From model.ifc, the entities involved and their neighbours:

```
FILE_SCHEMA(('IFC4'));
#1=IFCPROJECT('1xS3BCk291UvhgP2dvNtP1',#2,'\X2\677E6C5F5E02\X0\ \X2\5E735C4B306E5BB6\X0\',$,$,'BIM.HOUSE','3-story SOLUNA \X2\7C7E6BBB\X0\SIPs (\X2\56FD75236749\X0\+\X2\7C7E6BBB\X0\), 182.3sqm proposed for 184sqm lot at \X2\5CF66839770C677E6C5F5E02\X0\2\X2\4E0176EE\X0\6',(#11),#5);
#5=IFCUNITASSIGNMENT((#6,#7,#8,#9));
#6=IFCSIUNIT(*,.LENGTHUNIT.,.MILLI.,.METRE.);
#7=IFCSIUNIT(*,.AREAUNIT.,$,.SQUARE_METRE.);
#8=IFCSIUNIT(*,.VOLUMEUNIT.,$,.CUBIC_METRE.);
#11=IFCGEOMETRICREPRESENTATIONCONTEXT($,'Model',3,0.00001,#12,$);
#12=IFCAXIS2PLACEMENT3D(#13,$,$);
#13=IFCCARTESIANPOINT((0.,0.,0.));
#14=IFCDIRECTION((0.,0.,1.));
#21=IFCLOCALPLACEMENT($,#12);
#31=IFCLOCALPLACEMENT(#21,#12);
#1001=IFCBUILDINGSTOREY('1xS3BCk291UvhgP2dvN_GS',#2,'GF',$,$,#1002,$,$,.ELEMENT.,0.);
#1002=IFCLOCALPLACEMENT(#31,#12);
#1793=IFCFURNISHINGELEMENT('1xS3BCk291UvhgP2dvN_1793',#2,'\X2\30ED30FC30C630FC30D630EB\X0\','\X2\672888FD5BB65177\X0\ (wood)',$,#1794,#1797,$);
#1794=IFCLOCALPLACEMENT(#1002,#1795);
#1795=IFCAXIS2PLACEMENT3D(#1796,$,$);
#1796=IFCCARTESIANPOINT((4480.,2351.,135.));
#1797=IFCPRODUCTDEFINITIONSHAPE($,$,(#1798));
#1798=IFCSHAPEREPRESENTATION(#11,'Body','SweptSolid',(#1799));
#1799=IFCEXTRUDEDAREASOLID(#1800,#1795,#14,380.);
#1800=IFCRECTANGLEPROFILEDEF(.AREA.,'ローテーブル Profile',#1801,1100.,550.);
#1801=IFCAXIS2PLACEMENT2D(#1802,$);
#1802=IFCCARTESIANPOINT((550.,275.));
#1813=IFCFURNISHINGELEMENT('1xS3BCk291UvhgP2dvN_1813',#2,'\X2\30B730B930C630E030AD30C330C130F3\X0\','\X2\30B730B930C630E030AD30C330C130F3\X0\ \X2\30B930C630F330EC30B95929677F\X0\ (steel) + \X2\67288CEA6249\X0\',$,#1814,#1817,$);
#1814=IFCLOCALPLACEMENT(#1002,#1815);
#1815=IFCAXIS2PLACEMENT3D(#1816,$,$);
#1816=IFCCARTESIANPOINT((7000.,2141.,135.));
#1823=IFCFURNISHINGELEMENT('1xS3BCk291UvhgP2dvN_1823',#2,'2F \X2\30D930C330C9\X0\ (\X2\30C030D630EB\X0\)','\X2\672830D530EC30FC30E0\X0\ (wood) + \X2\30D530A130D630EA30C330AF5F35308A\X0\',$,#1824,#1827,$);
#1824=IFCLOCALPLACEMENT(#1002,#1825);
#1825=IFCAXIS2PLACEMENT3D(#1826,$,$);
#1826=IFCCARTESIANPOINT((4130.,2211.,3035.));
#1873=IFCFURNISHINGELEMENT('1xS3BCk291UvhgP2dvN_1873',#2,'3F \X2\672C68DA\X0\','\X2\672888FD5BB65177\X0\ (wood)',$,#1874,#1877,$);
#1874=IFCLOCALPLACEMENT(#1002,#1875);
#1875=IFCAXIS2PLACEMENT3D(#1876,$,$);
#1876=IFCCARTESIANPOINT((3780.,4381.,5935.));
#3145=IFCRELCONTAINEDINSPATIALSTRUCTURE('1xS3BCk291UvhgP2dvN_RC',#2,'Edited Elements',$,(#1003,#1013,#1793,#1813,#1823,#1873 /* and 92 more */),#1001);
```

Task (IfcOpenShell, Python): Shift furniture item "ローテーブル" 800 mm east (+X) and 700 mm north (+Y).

```python
import ifcopenshell
import ifcopenshell.api.geometry
import ifcopenshell.util.placement
import ifcopenshell.util.unit

model = ifcopenshell.open("model.ifc")
unit_scale = ifcopenshell.util.unit.calculate_unit_scale(model)

item = model.by_guid("1xS3BCk291UvhgP2dvN_1793")
matrix = ifcopenshell.util.placement.get_local_placement(item.ObjectPlacement)
matrix[0, 3] += 0.8 / unit_scale
matrix[1, 3] += 0.7 / unit_scale
ifcopenshell.api.geometry.edit_object_placement(model, product=item, matrix=matrix, is_si=False)

print(ifcopenshell.util.placement.get_local_placement(item.ObjectPlacement).round(3) + 0.0)

model.write("model_edited.ifc")
```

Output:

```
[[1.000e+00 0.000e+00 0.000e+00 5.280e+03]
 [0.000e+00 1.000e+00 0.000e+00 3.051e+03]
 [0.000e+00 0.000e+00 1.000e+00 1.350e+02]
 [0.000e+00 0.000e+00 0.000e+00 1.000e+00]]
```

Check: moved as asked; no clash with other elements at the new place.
